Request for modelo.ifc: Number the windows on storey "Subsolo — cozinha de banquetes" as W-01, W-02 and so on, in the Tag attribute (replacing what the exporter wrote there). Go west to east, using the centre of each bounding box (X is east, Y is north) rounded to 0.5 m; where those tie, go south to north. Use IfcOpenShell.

First a look at what the model holds.

```python
import ifcopenshell
import ifcopenshell.util.element
import ifcopenshell.util.placement

model = ifcopenshell.open("modelo.ifc")
print(model.schema)
storey = next(s for s in model.by_type("IfcBuildingStorey") if s.Name == "Subsolo — cozinha de banquetes")
windows = [e for e in ifcopenshell.util.element.get_decomposition(storey) if e.is_a("IfcWindow")]
for e in sorted(windows, key=lambda e: e.id()):
    origin = ifcopenshell.util.placement.get_local_placement(e.ObjectPlacement)[:3, 3]
    print(e.id(), e.Tag, e.Name, origin.round(2) + 0.0, sep=" | ")
```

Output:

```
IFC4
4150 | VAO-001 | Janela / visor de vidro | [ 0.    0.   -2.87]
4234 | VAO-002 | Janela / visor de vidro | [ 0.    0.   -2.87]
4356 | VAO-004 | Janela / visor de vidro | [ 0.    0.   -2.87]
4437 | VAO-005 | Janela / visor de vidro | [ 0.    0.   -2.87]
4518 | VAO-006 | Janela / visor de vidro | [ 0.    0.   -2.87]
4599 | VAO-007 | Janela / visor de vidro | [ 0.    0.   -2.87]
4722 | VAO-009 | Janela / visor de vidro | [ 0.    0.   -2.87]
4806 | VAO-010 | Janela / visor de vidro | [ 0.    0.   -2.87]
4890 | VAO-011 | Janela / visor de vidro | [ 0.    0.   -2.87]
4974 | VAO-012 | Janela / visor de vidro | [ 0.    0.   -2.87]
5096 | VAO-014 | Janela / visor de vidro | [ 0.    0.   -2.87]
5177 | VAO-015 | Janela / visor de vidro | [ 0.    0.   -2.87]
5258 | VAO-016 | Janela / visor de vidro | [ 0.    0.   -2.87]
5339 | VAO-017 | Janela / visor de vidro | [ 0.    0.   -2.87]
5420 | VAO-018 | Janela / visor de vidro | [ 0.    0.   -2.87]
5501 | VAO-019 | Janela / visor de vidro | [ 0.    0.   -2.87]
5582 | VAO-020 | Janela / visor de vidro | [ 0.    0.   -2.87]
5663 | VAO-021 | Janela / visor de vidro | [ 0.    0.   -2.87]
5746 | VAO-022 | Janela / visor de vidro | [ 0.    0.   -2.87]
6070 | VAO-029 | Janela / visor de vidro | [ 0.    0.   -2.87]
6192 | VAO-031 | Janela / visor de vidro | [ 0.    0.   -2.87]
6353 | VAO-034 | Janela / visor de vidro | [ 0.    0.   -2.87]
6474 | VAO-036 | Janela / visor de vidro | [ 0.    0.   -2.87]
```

```python
import ifcopenshell
import ifcopenshell.geom
import ifcopenshell.util.element
import ifcopenshell.util.shape

model = ifcopenshell.open("modelo.ifc")
settings = ifcopenshell.geom.settings()
settings.set("use-world-coords", True)


def centre(element):
    shape = ifcopenshell.geom.create_shape(settings, element)
    return ifcopenshell.util.shape.get_bbox_centroid(shape.geometry)


storey = next(s for s in model.by_type("IfcBuildingStorey") if s.Name == "Subsolo — cozinha de banquetes")
windows = [e for e in ifcopenshell.util.element.get_decomposition(storey) if e.is_a("IfcWindow")]

# Insertion points can sit at a corner or the storey origin, so sort by the geometry (in metres).
centres = {e: centre(e) for e in windows}
windows.sort(key=lambda e: (round(centres[e][0] / 0.5), centres[e][1]))

for i, e in enumerate(windows, start=1):
    number = f"W-{i:02d}"
    e.Tag = number
    print(e.id(), number)

model.write("modelo_v2.ifc")
```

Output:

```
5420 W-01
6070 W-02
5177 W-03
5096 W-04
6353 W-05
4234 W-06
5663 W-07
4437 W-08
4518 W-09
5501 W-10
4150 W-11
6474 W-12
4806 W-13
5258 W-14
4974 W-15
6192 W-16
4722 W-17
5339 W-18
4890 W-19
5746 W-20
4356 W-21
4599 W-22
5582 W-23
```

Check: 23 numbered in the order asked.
